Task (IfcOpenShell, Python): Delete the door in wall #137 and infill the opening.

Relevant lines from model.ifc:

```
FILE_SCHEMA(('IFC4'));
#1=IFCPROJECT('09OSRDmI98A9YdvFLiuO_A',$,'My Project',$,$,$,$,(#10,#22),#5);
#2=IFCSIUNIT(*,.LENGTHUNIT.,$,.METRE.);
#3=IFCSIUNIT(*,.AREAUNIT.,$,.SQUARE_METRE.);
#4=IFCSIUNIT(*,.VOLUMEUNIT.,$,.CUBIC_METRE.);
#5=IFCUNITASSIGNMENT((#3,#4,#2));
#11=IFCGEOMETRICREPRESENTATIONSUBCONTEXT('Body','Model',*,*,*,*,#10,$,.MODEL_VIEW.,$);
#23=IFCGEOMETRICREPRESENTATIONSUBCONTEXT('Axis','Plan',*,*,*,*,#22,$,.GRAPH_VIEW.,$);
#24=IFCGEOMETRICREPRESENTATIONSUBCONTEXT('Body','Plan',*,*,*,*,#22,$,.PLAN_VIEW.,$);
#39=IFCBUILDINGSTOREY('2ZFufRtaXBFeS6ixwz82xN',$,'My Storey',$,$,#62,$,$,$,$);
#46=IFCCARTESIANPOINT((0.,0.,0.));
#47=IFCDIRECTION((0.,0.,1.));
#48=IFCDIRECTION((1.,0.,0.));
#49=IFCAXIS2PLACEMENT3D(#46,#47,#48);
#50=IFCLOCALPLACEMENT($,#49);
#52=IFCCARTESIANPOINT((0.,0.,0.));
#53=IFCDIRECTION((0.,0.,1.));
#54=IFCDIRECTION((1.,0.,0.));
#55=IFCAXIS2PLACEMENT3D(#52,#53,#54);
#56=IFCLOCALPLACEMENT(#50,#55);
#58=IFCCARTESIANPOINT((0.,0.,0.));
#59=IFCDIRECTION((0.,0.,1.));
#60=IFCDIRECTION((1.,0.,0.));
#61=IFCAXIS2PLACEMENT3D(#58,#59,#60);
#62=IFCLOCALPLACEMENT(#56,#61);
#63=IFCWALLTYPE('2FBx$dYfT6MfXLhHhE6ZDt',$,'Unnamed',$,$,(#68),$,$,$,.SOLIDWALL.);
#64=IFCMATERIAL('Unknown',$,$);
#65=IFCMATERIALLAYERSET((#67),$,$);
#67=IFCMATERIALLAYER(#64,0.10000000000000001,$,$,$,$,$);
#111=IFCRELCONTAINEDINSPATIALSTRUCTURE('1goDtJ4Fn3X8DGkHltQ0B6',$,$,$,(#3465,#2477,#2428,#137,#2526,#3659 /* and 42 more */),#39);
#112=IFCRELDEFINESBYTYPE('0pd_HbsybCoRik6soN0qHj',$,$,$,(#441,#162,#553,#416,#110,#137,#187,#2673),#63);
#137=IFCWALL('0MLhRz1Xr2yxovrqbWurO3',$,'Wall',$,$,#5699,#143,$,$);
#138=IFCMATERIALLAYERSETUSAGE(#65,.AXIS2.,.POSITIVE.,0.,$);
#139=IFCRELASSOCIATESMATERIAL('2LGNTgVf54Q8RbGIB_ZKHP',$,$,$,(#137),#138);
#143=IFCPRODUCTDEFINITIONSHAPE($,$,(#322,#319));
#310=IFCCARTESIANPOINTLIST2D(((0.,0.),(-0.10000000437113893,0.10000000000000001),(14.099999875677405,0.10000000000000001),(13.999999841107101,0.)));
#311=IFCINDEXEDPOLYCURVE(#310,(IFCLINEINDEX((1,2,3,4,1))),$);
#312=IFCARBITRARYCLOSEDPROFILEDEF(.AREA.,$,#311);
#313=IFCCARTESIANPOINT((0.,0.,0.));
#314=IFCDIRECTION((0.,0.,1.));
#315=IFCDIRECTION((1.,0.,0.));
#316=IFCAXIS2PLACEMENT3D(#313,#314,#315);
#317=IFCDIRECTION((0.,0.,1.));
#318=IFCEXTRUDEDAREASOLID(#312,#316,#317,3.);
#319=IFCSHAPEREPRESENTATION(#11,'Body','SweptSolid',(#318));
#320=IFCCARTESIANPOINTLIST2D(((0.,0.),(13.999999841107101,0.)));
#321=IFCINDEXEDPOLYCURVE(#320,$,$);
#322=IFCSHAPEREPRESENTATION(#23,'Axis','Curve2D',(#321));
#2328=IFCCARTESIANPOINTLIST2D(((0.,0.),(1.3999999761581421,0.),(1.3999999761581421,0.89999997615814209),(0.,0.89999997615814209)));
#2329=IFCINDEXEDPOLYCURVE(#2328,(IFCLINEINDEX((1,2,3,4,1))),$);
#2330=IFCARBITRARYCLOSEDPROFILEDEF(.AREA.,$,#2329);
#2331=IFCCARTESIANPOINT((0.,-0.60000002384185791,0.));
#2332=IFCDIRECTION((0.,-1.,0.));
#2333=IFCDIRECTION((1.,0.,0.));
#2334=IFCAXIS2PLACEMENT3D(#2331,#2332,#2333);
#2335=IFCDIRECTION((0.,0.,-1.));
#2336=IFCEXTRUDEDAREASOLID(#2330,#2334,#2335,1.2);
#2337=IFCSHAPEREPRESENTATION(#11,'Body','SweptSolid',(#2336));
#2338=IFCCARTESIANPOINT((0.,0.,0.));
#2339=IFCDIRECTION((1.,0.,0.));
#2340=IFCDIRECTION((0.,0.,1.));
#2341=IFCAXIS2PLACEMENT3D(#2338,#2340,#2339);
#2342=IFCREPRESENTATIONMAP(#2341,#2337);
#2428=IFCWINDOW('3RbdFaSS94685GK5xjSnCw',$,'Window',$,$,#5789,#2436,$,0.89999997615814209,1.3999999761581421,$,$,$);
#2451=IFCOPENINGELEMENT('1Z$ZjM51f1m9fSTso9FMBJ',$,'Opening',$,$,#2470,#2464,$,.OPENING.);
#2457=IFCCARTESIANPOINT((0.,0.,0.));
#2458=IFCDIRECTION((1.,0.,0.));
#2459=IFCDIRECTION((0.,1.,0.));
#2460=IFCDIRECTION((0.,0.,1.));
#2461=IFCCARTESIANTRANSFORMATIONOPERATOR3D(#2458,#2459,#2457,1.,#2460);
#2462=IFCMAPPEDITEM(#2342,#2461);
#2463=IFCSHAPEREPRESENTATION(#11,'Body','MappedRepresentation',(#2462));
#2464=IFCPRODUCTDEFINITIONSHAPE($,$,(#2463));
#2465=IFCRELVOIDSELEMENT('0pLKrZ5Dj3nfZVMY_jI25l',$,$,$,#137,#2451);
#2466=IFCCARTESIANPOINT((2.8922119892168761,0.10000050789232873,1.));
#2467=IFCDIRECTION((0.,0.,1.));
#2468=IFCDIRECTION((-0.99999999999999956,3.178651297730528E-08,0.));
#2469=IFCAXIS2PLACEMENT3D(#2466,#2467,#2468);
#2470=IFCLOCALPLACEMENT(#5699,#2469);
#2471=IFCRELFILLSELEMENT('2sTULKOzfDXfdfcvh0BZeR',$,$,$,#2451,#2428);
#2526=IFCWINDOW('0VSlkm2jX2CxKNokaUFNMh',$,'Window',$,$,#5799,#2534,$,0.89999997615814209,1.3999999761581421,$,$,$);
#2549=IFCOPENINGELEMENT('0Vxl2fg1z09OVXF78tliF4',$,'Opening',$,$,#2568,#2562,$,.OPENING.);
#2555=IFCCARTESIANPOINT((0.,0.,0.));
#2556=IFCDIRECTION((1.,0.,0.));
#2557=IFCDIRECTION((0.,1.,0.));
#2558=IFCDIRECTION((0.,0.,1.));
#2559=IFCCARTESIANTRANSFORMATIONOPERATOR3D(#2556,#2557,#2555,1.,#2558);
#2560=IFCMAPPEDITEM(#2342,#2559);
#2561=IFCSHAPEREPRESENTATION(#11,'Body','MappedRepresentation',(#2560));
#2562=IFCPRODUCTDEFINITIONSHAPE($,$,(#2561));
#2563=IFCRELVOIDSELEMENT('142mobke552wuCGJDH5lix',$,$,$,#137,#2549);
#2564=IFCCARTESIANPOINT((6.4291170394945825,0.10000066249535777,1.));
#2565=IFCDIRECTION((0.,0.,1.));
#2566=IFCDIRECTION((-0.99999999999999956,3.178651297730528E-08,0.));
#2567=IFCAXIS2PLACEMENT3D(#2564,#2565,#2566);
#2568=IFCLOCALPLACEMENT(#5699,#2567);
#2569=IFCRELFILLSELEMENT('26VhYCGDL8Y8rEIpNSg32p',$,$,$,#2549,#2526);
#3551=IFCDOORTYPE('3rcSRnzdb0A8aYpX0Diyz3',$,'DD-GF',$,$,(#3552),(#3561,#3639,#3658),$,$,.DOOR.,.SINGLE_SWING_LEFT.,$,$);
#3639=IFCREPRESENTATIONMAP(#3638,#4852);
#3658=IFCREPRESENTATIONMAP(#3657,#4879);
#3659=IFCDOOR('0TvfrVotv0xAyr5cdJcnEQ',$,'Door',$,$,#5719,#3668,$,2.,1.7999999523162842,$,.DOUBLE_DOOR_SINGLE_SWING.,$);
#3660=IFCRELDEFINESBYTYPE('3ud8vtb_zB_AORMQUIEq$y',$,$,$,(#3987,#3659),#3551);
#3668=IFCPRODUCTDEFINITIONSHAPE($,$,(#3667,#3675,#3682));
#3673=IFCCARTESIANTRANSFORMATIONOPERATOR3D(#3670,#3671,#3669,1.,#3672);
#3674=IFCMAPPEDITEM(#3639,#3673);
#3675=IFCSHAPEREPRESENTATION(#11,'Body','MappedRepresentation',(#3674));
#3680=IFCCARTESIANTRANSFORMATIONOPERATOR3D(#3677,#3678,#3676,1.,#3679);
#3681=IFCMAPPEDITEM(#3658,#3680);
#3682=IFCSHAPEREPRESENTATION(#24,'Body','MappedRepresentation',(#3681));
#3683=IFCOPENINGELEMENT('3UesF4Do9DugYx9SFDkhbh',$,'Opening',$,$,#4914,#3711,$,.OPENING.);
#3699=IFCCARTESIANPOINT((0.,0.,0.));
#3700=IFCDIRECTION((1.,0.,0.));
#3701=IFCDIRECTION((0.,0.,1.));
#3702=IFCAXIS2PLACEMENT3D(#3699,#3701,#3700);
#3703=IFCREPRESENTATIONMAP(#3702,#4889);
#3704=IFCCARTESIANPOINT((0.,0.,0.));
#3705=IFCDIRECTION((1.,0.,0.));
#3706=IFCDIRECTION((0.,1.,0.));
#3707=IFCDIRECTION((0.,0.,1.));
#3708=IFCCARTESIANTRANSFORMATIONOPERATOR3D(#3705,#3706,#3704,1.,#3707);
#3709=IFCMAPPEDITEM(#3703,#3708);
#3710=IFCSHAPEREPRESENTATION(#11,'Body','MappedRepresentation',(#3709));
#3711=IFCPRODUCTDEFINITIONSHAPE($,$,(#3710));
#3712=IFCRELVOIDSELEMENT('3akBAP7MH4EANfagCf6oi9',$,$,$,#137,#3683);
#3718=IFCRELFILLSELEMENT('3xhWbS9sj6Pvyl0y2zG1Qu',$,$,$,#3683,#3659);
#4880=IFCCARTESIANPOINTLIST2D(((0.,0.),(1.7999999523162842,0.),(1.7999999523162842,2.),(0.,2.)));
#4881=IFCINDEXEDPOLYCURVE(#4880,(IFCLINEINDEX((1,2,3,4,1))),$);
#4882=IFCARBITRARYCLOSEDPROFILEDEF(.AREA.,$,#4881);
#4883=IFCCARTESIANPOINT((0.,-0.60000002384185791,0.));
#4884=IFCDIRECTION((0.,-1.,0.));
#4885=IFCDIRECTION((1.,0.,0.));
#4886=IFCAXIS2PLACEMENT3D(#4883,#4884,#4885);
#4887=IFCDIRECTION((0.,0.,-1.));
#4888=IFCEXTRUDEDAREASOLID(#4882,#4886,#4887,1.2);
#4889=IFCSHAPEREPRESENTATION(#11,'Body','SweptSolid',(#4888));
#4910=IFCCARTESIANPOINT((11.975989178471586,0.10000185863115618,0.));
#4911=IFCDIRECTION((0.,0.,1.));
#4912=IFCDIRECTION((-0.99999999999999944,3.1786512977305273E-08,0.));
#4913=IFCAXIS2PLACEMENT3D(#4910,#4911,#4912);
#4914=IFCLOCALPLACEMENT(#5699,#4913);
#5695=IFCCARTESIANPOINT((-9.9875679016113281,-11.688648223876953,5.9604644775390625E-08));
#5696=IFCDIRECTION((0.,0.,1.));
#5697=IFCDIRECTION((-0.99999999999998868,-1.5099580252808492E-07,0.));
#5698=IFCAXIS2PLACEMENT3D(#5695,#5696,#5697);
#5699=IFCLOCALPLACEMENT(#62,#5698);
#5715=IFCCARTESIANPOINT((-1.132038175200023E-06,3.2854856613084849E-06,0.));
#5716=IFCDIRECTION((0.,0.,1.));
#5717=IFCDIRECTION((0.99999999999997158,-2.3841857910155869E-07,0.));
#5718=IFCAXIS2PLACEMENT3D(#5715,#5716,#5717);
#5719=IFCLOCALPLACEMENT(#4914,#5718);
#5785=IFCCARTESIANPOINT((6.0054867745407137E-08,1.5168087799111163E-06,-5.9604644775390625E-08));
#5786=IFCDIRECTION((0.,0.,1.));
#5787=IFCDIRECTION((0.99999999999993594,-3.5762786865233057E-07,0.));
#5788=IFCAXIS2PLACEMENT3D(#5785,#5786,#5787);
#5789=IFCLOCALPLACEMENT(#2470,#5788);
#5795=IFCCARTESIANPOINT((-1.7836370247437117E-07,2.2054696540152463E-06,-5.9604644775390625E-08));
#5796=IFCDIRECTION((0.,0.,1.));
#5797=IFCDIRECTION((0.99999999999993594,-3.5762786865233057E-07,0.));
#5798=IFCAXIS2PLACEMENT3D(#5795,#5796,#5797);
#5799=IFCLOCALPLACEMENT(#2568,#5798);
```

```python
import ifcopenshell
import ifcopenshell.api.feature
import ifcopenshell.api.root
import ifcopenshell.geom
import ifcopenshell.util.shape

model = ifcopenshell.open("model.ifc")
settings = ifcopenshell.geom.settings()


def volume(element):
    """Net volume in cubic metres, openings subtracted."""
    shape = ifcopenshell.geom.create_shape(settings, element)
    return ifcopenshell.util.shape.get_volume(shape.geometry)


door = model.by_guid("0TvfrVotv0xAyr5cdJcnEQ")
opening = door.FillsVoids[0].RelatingOpeningElement
wall = opening.VoidsElements[0].RelatingBuildingElement
before = volume(wall)

ifcopenshell.api.root.remove_product(model, product=door)
ifcopenshell.api.feature.remove_feature(model, feature=opening)

after = volume(wall)

print(f"wall volume {before:.3f} -> {after:.3f} m3")

model.write("model_rev.ifc")
```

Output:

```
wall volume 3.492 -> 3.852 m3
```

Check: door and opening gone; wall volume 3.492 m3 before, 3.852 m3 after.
